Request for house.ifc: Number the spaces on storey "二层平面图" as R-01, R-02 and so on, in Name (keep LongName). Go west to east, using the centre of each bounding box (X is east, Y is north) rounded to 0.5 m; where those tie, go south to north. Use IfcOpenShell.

First a look at what the model holds.

```python
import ifcopenshell
import ifcopenshell.util.element
import ifcopenshell.util.placement

model = ifcopenshell.open("house.ifc")
print(model.schema)
storey = next(s for s in model.by_type("IfcBuildingStorey") if s.Name == "二层平面图")
spaces = [e for e in ifcopenshell.util.element.get_decomposition(storey) if e.is_a("IfcSpace")]
for e in sorted(spaces, key=lambda e: e.id()):
    origin = ifcopenshell.util.placement.get_local_placement(e.ObjectPlacement)[:3, 3]
    print(e.id(), e.Name, e.LongName, origin.round(2) + 0.0, sep=" | ")
```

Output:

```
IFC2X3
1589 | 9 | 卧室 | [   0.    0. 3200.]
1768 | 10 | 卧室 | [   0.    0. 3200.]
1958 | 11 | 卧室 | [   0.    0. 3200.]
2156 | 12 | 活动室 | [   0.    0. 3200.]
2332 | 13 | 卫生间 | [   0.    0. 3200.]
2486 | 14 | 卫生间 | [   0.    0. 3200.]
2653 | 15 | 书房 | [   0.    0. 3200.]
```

```python
import ifcopenshell
import ifcopenshell.geom
import ifcopenshell.util.element
import ifcopenshell.util.shape

model = ifcopenshell.open("house.ifc")
settings = ifcopenshell.geom.settings()
settings.set("use-world-coords", True)


def centre(element):
    shape = ifcopenshell.geom.create_shape(settings, element)
    return ifcopenshell.util.shape.get_bbox_centroid(shape.geometry)


storey = next(s for s in model.by_type("IfcBuildingStorey") if s.Name == "二层平面图")
spaces = [e for e in ifcopenshell.util.element.get_decomposition(storey) if e.is_a("IfcSpace")]

# Insertion points can sit at a corner or the storey origin, so sort by the geometry (in metres).
centres = {e: centre(e) for e in spaces}
spaces.sort(key=lambda e: (round(centres[e][0] / 0.5), centres[e][1]))

for i, e in enumerate(spaces, start=1):
    number = f"R-{i:02d}"
    e.Name = number
    print(e.id(), number)

model.write("house_v2.ifc")
```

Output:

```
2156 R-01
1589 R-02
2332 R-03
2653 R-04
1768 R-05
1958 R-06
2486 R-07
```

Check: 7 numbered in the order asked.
